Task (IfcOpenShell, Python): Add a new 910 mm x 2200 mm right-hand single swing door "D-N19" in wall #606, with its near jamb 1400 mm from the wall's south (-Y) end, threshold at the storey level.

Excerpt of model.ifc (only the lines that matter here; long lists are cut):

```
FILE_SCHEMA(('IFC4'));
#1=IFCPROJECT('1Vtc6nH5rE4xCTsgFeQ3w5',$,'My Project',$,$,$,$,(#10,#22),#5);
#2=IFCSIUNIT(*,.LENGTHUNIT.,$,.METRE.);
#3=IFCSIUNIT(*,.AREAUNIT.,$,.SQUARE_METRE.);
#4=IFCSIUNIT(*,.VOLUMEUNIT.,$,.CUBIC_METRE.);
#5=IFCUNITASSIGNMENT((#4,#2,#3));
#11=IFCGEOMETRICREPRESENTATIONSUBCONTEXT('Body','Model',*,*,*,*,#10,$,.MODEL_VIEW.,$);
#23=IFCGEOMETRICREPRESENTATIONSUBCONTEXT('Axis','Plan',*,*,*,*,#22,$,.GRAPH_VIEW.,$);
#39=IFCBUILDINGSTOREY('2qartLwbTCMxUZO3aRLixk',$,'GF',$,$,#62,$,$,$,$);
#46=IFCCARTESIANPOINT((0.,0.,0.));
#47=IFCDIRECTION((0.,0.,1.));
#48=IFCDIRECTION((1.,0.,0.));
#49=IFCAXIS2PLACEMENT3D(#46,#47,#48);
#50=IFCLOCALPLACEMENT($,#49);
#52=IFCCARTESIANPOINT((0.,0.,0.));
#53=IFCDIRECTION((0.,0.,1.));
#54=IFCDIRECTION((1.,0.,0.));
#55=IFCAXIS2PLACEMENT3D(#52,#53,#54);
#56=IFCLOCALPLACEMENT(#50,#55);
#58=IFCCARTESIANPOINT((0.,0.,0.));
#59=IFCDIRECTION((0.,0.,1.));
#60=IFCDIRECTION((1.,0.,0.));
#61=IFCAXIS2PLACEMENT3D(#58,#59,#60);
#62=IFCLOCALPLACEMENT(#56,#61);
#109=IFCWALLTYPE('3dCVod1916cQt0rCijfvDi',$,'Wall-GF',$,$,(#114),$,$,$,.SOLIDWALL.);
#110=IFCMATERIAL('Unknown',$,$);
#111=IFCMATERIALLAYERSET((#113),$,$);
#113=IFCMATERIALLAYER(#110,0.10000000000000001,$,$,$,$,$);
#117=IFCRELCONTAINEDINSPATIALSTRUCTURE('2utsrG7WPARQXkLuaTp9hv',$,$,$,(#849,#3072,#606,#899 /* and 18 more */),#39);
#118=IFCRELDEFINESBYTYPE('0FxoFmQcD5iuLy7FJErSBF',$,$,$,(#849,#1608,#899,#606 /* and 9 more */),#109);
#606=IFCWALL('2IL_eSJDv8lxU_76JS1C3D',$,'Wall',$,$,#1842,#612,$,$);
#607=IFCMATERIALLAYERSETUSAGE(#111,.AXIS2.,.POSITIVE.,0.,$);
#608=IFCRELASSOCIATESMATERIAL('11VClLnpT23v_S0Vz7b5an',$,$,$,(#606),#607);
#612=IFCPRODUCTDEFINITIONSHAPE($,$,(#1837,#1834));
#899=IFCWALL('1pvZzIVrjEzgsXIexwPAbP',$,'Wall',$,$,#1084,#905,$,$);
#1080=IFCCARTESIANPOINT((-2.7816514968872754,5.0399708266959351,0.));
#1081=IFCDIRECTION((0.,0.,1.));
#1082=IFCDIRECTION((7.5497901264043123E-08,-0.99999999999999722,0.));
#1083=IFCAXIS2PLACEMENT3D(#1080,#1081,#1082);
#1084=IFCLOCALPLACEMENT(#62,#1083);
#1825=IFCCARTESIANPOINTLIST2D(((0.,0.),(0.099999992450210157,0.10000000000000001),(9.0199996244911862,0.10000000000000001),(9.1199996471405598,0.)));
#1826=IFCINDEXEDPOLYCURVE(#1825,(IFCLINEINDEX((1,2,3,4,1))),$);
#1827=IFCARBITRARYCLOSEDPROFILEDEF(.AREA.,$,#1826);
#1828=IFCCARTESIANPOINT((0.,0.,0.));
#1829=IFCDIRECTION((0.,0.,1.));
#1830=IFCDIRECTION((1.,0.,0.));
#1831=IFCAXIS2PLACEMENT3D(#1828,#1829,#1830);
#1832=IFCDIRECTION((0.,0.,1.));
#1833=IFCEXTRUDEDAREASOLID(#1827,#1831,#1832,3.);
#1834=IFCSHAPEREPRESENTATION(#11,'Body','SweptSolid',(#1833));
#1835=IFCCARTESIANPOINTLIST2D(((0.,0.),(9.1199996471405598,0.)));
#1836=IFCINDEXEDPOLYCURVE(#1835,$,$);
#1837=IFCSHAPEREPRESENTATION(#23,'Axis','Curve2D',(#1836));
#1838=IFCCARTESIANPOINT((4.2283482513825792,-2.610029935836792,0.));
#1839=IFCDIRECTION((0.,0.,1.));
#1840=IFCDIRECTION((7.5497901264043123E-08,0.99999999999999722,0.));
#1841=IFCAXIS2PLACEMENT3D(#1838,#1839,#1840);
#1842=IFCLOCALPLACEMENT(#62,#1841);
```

```python
import numpy as np
import ifcopenshell
import ifcopenshell.api.feature
import ifcopenshell.api.geometry
import ifcopenshell.api.root
import ifcopenshell.api.spatial
import ifcopenshell.geom
import ifcopenshell.util.element
import ifcopenshell.util.placement
import ifcopenshell.util.representation
import ifcopenshell.util.shape
import ifcopenshell.util.unit

model = ifcopenshell.open("model.ifc")
unit_scale = ifcopenshell.util.unit.calculate_unit_scale(model)
settings = ifcopenshell.geom.settings()


def volume(element):
    """Net volume in cubic metres, openings subtracted."""
    shape = ifcopenshell.geom.create_shape(settings, element)
    return ifcopenshell.util.shape.get_volume(shape.geometry)


wall = model.by_guid("2IL_eSJDv8lxU_76JS1C3D")
storey = ifcopenshell.util.element.get_container(wall, ifc_class="IfcBuildingStorey")
context = ifcopenshell.util.representation.get_context(model, "Model", "Body", "MODEL_VIEW")
before = volume(wall)

width, height, from_end, sill = 0.91, 2.2, 1.4, 0.0  # metres

# The wall runs along its own X axis, and the end named is its -X end.
wall_shape = ifcopenshell.geom.create_shape(settings, wall)
x, y, z = ifcopenshell.util.shape.get_vertices(wall_shape.geometry).T
start = x.min() + from_end
face, thickness = float(y.min()), float(y.max() - y.min())
wall_matrix = ifcopenshell.util.placement.get_local_placement(wall.ObjectPlacement)
level = ifcopenshell.util.placement.get_local_placement(storey.ObjectPlacement)[2, 3]


def in_wall(x, y):
    """Placement at x, y metres in the wall's axes, at sill height."""
    matrix = wall_matrix.copy()
    matrix[:, 3] = wall_matrix @ np.array([x / unit_scale, y / unit_scale, 0.0, 1.0])
    matrix[2, 3] = level + sill / unit_scale
    return matrix


# Opening: a box that overshoots both wall faces by 50 mm.
opening = ifcopenshell.api.root.create_entity(model, ifc_class="IfcOpeningElement", predefined_type="OPENING")
box = ifcopenshell.api.geometry.add_wall_representation(
    model, context=context, length=width, height=height, thickness=thickness + 0.1
)
ifcopenshell.api.geometry.assign_representation(model, product=opening, representation=box)
ifcopenshell.api.geometry.edit_object_placement(model, product=opening, matrix=in_wall(start, face - 0.05), is_si=False)
ifcopenshell.api.feature.add_feature(model, feature=opening, element=wall)

door = ifcopenshell.api.root.create_entity(model, ifc_class="IfcDoor", name="D-N19", predefined_type="DOOR")
door.OverallWidth, door.OverallHeight = width / unit_scale, height / unit_scale
door.OperationType = "SINGLE_SWING_RIGHT"
body = ifcopenshell.api.geometry.add_door_representation(
    model,
    context=context,
    overall_width=door.OverallWidth,
    overall_height=door.OverallHeight,
    operation_type="SINGLE_SWING_RIGHT",
    lining_properties={"LiningDepth": thickness / unit_scale, "ThresholdDepth": thickness / unit_scale},
)
ifcopenshell.api.geometry.assign_representation(model, product=door, representation=body)
ifcopenshell.api.spatial.assign_container(model, products=[door], relating_structure=storey)
ifcopenshell.api.feature.add_filling(model, opening=opening, element=door)

# The lining spans the wall, so the door starts at the wall face.
ifcopenshell.api.geometry.edit_object_placement(model, product=door, matrix=in_wall(start, face), is_si=False)

after = volume(wall)

print(f"wall volume {before:.3f} -> {after:.3f} m3")

model.write("model_updated.ifc")
```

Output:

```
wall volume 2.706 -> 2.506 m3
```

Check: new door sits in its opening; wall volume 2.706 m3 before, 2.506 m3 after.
